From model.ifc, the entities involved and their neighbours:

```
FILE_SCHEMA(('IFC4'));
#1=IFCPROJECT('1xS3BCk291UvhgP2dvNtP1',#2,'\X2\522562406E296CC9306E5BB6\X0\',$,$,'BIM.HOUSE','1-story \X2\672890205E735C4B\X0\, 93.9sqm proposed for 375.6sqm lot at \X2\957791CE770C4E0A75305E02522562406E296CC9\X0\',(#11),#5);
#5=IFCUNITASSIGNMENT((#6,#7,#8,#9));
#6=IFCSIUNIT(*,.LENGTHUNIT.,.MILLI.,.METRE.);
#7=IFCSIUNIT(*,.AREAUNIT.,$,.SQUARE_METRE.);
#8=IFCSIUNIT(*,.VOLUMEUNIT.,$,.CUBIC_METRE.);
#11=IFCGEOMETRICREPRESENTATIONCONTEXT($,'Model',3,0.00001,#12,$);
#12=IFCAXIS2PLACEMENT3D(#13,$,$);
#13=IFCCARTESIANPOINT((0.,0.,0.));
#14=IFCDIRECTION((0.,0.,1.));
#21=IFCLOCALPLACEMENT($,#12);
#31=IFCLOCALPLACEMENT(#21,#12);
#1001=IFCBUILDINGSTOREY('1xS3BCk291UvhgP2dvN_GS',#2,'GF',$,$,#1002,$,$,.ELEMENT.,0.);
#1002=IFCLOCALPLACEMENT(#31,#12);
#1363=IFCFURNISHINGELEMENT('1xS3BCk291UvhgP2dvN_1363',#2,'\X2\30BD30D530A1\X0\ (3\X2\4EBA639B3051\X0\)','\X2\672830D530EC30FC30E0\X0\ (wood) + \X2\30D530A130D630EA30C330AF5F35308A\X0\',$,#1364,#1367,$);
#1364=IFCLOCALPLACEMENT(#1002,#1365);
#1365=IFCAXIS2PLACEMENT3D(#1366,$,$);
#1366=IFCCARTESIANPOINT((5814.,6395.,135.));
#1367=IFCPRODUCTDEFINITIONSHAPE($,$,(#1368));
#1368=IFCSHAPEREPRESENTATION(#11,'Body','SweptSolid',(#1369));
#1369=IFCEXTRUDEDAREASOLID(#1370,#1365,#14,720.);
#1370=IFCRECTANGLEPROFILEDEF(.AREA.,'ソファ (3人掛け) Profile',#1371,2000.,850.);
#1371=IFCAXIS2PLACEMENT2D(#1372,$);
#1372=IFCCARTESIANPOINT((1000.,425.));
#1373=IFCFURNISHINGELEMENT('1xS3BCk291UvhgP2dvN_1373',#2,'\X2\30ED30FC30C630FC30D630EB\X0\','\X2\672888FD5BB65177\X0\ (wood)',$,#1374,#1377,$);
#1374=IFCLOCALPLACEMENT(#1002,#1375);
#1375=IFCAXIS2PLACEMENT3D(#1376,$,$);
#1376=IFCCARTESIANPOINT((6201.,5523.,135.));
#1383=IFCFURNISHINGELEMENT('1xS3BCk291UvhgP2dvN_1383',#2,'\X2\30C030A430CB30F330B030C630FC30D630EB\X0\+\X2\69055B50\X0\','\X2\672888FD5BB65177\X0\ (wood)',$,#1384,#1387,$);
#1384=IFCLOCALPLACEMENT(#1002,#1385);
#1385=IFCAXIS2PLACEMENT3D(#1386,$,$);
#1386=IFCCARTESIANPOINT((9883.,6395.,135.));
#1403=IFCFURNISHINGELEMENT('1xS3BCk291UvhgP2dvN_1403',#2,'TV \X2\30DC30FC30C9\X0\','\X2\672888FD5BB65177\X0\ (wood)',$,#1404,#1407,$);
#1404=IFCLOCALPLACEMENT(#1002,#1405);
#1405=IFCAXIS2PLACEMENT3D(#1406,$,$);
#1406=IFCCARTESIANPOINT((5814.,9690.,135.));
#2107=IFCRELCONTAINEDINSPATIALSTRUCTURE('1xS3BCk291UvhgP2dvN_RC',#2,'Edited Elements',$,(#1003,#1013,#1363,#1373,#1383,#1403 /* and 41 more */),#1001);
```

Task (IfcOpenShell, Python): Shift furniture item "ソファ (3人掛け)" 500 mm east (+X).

```python
import ifcopenshell
import ifcopenshell.api.geometry
import ifcopenshell.util.placement
import ifcopenshell.util.unit

model = ifcopenshell.open("model.ifc")
unit_scale = ifcopenshell.util.unit.calculate_unit_scale(model)

item = model.by_guid("1xS3BCk291UvhgP2dvN_1363")
matrix = ifcopenshell.util.placement.get_local_placement(item.ObjectPlacement)
matrix[0, 3] += 0.5 / unit_scale
ifcopenshell.api.geometry.edit_object_placement(model, product=item, matrix=matrix, is_si=False)

print(ifcopenshell.util.placement.get_local_placement(item.ObjectPlacement).round(3) + 0.0)

model.write("model_rev.ifc")
```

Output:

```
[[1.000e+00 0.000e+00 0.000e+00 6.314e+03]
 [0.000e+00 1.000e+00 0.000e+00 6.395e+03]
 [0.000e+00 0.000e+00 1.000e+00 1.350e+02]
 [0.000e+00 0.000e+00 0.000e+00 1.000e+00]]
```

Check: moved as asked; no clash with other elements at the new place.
